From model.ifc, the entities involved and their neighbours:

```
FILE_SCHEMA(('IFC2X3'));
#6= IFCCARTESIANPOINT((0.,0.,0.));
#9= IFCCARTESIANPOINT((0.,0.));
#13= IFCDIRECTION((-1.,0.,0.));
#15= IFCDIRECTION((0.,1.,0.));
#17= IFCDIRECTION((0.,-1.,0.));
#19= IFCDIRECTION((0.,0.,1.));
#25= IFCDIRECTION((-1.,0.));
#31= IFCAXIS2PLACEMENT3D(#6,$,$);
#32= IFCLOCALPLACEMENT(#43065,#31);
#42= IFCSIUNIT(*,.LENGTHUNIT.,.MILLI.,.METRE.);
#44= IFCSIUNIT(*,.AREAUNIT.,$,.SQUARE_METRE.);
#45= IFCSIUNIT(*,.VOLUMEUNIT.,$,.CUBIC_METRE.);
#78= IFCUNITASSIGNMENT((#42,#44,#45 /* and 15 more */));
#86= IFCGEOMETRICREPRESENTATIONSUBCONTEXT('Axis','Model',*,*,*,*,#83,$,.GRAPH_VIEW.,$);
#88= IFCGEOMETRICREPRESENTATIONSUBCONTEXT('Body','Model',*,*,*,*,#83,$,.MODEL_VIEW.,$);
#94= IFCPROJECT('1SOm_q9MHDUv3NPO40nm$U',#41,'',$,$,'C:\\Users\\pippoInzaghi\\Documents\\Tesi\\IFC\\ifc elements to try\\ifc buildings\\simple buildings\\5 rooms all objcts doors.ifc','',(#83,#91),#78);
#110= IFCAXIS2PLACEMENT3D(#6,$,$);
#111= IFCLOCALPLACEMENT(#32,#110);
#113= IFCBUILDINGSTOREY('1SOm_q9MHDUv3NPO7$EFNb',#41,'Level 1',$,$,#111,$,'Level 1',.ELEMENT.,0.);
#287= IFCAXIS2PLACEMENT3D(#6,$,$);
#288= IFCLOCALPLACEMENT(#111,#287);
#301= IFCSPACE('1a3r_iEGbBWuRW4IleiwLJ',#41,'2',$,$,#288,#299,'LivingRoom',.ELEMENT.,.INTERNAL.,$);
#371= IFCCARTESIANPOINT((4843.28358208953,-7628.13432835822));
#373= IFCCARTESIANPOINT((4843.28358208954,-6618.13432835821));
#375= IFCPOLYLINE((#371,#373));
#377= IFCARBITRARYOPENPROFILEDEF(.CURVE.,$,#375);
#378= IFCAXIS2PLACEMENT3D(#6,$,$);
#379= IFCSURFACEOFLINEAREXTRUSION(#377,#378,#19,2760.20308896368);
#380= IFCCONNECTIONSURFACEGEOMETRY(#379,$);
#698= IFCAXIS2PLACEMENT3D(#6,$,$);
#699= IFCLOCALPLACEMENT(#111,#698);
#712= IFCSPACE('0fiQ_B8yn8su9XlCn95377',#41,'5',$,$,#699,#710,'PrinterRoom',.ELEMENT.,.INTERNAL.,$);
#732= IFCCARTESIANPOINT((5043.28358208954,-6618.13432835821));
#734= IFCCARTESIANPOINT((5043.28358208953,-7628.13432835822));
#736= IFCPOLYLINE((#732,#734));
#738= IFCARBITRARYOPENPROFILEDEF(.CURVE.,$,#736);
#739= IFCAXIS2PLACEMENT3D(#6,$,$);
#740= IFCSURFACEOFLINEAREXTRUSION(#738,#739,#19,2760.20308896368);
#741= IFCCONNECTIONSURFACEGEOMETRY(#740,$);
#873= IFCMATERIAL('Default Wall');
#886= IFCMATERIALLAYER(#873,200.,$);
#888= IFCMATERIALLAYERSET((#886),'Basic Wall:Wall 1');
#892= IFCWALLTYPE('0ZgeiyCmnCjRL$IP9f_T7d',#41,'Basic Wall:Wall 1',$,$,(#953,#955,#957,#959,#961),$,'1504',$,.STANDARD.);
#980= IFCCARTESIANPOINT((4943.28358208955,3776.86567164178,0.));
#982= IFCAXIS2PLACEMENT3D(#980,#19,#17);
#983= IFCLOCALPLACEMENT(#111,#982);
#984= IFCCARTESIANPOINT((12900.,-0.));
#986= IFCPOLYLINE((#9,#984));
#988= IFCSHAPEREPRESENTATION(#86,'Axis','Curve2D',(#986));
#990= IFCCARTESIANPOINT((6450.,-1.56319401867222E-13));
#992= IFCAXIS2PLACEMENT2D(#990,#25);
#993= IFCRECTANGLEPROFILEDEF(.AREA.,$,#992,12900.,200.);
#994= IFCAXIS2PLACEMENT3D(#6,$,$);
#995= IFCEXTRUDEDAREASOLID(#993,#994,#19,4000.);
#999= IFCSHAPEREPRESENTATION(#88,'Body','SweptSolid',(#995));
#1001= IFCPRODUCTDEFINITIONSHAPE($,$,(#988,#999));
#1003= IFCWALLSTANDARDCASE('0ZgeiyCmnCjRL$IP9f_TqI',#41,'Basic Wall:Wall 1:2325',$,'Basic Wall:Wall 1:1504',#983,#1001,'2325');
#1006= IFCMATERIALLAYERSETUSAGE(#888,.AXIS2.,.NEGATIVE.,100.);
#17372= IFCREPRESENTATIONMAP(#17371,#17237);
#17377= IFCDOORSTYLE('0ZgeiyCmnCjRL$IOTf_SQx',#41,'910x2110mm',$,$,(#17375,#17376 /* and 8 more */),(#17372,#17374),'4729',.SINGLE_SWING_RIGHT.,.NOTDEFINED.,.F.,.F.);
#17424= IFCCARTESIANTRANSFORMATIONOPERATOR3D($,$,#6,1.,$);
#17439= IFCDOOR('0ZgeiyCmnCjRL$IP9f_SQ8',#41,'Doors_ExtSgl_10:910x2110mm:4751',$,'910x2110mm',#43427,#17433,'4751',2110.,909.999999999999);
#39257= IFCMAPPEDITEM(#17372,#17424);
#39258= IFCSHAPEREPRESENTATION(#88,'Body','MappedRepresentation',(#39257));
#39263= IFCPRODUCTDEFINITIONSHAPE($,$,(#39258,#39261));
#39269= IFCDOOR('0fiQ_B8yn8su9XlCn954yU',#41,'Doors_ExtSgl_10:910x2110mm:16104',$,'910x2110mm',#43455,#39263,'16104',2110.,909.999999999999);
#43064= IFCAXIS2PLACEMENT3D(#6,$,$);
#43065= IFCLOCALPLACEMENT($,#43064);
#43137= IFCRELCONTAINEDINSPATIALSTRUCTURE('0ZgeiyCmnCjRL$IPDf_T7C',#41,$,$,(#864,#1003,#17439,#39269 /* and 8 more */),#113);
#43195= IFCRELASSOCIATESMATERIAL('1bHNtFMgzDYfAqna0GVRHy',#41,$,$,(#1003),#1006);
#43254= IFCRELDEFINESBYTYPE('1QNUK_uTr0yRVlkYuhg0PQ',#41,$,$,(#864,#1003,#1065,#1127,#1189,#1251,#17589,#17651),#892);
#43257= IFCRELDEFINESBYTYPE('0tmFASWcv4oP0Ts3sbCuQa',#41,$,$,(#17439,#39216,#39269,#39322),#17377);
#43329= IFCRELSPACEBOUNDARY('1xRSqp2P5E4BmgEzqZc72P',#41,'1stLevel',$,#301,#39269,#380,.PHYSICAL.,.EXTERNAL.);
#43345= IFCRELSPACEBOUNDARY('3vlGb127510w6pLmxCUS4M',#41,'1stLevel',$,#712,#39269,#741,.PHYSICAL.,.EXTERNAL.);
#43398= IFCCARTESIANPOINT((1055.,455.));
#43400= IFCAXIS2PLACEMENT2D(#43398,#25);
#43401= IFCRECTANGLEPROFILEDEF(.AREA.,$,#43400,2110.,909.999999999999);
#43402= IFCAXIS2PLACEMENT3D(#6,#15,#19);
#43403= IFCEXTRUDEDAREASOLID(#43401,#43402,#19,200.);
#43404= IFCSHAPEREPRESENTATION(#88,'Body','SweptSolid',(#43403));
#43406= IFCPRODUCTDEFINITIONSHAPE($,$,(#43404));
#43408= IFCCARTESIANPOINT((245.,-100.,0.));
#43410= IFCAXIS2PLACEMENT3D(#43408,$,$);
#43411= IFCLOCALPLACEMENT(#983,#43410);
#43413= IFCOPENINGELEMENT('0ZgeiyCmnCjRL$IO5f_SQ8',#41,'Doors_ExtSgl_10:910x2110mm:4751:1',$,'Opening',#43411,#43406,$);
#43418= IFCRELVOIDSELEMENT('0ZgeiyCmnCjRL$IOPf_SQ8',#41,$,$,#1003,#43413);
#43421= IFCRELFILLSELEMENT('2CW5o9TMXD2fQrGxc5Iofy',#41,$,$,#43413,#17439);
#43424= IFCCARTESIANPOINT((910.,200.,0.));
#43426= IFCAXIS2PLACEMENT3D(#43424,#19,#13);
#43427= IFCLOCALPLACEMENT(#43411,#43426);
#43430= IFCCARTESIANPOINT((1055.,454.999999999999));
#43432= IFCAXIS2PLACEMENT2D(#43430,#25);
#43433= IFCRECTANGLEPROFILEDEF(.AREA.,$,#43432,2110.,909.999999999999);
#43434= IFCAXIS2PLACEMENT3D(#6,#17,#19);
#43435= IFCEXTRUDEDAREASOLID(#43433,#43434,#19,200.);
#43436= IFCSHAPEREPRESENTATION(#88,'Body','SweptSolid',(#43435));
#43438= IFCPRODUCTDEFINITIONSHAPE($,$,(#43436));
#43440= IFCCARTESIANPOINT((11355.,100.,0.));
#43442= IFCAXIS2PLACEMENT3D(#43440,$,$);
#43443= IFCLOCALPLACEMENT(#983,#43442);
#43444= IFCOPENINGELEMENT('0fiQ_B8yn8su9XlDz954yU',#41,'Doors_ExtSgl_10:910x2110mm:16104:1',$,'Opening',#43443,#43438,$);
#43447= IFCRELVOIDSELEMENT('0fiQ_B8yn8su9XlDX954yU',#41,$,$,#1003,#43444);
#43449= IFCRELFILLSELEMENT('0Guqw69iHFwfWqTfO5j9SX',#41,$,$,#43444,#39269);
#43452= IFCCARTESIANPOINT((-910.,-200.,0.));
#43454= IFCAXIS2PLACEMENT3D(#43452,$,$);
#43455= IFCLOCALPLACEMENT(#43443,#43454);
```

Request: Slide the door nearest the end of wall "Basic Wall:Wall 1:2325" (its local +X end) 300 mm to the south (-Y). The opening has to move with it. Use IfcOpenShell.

```python
import numpy as np
import ifcopenshell
import ifcopenshell.api.geometry
import ifcopenshell.util.placement
import ifcopenshell.util.unit

model = ifcopenshell.open("model.ifc")
unit_scale = ifcopenshell.util.unit.calculate_unit_scale(model)

door = model.by_id(39269)
opening = door.FillsVoids[0].RelatingOpeningElement
wall = opening.VoidsElements[0].RelatingBuildingElement

wall_matrix = ifcopenshell.util.placement.get_local_placement(wall.ObjectPlacement)
shift = wall_matrix[:3, 0] * 0.3 / unit_scale
before = ifcopenshell.util.placement.get_local_placement(door.ObjectPlacement)[:3, 3].copy()

# The door is placed relative to its opening, so it follows when the opening moves.
matrix = ifcopenshell.util.placement.get_local_placement(opening.ObjectPlacement)
matrix[:3, 3] += shift
ifcopenshell.api.geometry.edit_object_placement(
    model, product=opening, matrix=matrix, is_si=False, should_transform_children=True
)

# Space boundary surfaces are stored in each space's coordinates; move them too.
for rel in door.ProvidesBoundaries:
    if not rel.ConnectionGeometry:
        continue
    surface = rel.ConnectionGeometry.SurfaceOnRelatingElement
    space_matrix = ifcopenshell.util.placement.get_local_placement(rel.RelatingSpace.ObjectPlacement)
    point = np.array(surface.Position.Location.Coordinates) + space_matrix[:3, :3].T @ shift
    surface.Position = model.createIfcAxis2Placement3D(
        model.createIfcCartesianPoint(point.tolist()), surface.Position.Axis, surface.Position.RefDirection
    )

after = ifcopenshell.util.placement.get_local_placement(door.ObjectPlacement)[:3, 3]
print("door moved by", (after - before).round(3) + 0.0)

model.write("model_rev.ifc")
```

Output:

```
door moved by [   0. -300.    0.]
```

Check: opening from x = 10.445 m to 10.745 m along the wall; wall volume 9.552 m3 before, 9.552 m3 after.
